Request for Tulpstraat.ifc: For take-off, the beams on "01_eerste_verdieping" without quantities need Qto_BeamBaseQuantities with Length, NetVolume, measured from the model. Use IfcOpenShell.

First a look at what the model holds.

```python
import ifcopenshell
import ifcopenshell.util.element
import ifcopenshell.util.unit

model = ifcopenshell.open("Tulpstraat.ifc")
print(model.schema)
for unit_type in ("LENGTHUNIT", "AREAUNIT", "VOLUMEUNIT"):
    print(unit_type, ifcopenshell.util.unit.calculate_unit_scale(model, unit_type))
storey = next(s for s in model.by_type("IfcBuildingStorey") if s.Name == "01_eerste_verdieping")
beams = [e for e in ifcopenshell.util.element.get_decomposition(storey) if e.is_a("IfcBeam")]
for e in sorted(beams, key=lambda e: e.id()):
    print(e.id(), e.is_a(), e.Name, list(ifcopenshell.util.element.get_psets(e, qtos_only=True)), sep=" | ")
```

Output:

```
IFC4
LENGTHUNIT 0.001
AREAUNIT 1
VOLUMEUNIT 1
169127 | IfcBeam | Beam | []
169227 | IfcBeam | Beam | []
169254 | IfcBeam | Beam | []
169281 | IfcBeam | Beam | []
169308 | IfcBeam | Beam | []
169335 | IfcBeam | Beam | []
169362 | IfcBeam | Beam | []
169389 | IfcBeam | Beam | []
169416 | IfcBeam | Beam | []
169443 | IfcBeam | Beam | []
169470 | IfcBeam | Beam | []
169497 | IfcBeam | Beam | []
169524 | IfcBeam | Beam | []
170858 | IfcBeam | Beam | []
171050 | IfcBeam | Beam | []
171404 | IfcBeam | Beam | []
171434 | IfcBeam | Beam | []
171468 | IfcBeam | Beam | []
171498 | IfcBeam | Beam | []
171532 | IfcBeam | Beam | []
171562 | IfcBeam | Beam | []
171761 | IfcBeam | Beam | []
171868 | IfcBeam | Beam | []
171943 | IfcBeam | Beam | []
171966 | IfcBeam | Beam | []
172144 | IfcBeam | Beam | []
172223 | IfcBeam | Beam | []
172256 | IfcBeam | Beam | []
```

```python
import ifcopenshell
import ifcopenshell.api.pset
import ifcopenshell.geom
import ifcopenshell.util.element
import ifcopenshell.util.shape
import ifcopenshell.util.unit

model = ifcopenshell.open("Tulpstraat.ifc")
unit_scale = ifcopenshell.util.unit.calculate_unit_scale(model)
volume_scale = ifcopenshell.util.unit.calculate_unit_scale(model, "VOLUMEUNIT")
settings = ifcopenshell.geom.settings()

storey = next(s for s in model.by_type("IfcBuildingStorey") if s.Name == "01_eerste_verdieping")
beams = [e for e in ifcopenshell.util.element.get_decomposition(storey) if e.is_a("IfcBeam")]

for e in sorted(beams, key=lambda e: e.id()):
    if ifcopenshell.util.element.get_psets(e, qtos_only=True, should_inherit=False):
        continue
    # Geometry comes back in metres, in the element's own axes.
    shape = ifcopenshell.geom.create_shape(settings, e)
    values = {
        "Length": ifcopenshell.util.shape.get_max_xyz(shape.geometry) / unit_scale,
        "NetVolume": ifcopenshell.util.shape.get_volume(shape.geometry) / volume_scale,
    }
    qto = ifcopenshell.api.pset.add_qto(model, product=e, name="Qto_BeamBaseQuantities")
    ifcopenshell.api.pset.edit_qto(model, qto=qto, properties=values)
    print(e.id(), {k: round(v, 3) for k, v in values.items()})

model.write("Tulpstraat_rev.ifc")
```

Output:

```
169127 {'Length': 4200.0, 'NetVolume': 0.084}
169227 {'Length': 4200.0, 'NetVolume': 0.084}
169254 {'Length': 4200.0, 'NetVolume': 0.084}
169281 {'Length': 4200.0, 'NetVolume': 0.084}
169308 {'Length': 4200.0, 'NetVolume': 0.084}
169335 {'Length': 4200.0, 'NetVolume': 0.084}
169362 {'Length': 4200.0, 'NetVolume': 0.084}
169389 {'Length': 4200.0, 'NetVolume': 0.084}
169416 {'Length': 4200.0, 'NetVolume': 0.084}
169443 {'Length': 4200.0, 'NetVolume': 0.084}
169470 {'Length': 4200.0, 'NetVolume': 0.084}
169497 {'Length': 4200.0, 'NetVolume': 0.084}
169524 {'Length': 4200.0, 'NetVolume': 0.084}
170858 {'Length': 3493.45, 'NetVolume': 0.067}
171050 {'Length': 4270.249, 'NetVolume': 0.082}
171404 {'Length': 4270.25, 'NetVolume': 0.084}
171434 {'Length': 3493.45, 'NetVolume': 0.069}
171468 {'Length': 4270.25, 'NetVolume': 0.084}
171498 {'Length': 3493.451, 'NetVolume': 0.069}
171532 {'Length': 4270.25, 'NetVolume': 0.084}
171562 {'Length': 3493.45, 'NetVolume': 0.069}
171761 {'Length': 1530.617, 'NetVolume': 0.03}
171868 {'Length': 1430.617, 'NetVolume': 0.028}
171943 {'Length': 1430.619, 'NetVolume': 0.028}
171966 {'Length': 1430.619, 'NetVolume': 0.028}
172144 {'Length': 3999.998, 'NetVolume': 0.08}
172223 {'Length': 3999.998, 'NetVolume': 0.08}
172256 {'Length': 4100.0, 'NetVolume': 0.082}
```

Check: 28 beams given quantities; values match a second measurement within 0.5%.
